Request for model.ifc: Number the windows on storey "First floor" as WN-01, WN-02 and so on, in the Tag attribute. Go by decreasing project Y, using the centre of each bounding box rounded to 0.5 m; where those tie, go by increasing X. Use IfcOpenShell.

First a look at what the model holds.

```python
import ifcopenshell
import ifcopenshell.util.element
import ifcopenshell.util.placement

model = ifcopenshell.open("model.ifc")
print(model.schema)
storey = next(s for s in model.by_type("IfcBuildingStorey") if s.Name == "First floor")
windows = [e for e in ifcopenshell.util.element.get_decomposition(storey) if e.is_a("IfcWindow")]
for e in sorted(windows, key=lambda e: e.id()):
    origin = ifcopenshell.util.placement.get_local_placement(e.ObjectPlacement)[:3, 3]
    print(e.id(), e.Tag, e.Name, origin.round(2) + 0.0, sep=" | ")
```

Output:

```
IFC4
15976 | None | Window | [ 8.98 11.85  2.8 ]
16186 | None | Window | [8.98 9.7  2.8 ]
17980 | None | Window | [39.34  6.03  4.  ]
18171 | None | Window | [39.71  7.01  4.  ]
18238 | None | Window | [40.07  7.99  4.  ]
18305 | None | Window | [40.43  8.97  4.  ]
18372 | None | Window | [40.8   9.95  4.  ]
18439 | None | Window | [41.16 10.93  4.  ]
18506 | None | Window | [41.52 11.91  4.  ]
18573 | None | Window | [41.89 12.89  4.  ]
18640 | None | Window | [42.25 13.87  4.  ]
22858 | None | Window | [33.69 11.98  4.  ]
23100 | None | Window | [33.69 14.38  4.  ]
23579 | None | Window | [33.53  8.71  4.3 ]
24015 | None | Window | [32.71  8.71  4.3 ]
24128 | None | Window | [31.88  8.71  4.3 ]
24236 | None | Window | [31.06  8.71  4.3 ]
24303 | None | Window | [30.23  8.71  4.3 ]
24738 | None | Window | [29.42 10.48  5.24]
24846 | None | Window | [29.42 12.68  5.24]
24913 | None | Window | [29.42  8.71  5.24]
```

```python
import ifcopenshell
import ifcopenshell.geom
import ifcopenshell.util.element
import ifcopenshell.util.shape

model = ifcopenshell.open("model.ifc")
settings = ifcopenshell.geom.settings()
settings.set("use-world-coords", True)


def centre(element):
    shape = ifcopenshell.geom.create_shape(settings, element)
    return ifcopenshell.util.shape.get_bbox_centroid(shape.geometry)


storey = next(s for s in model.by_type("IfcBuildingStorey") if s.Name == "First floor")
windows = [e for e in ifcopenshell.util.element.get_decomposition(storey) if e.is_a("IfcWindow")]

# Insertion points can sit at a corner or the storey origin, so sort by the geometry (in metres).
centres = {e: centre(e) for e in windows}
windows.sort(key=lambda e: (-round(centres[e][1] / 0.5), centres[e][0]))

for i, e in enumerate(windows, start=1):
    number = f"WN-{i:02d}"
    e.Tag = number
    print(e.id(), number)

model.write("model_rev.ifc")
```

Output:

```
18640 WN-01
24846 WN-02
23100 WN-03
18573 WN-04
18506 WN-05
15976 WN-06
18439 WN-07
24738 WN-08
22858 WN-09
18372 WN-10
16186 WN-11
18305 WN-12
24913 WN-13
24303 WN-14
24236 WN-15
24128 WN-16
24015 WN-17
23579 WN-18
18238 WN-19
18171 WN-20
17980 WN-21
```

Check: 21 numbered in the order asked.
